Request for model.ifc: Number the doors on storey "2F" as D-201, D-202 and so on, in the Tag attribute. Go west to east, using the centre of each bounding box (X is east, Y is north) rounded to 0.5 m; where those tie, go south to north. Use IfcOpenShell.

First a look at what the model holds.

```python
import ifcopenshell
import ifcopenshell.util.element
import ifcopenshell.util.placement

model = ifcopenshell.open("model.ifc")
print(model.schema)
storey = next(s for s in model.by_type("IfcBuildingStorey") if s.Name == "2F")
doors = [e for e in ifcopenshell.util.element.get_decomposition(storey) if e.is_a("IfcDoor")]
for e in sorted(doors, key=lambda e: e.id()):
    origin = ifcopenshell.util.placement.get_local_placement(e.ObjectPlacement)[:3, 3]
    print(e.id(), e.Tag, e.Name, origin.round(2) + 0.0, sep=" | ")
```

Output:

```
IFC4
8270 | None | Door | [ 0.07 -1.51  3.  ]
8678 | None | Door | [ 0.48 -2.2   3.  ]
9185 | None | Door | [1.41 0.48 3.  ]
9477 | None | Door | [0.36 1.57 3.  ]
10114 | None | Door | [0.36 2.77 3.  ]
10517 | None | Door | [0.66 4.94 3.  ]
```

```python
import ifcopenshell
import ifcopenshell.geom
import ifcopenshell.util.element
import ifcopenshell.util.shape

model = ifcopenshell.open("model.ifc")
settings = ifcopenshell.geom.settings()
settings.set("use-world-coords", True)


def centre(element):
    shape = ifcopenshell.geom.create_shape(settings, element)
    return ifcopenshell.util.shape.get_bbox_centroid(shape.geometry)


storey = next(s for s in model.by_type("IfcBuildingStorey") if s.Name == "2F")
doors = [e for e in ifcopenshell.util.element.get_decomposition(storey) if e.is_a("IfcDoor")]

# Insertion points can sit at a corner or the storey origin, so sort by the geometry (in metres).
centres = {e: centre(e) for e in doors}
doors.sort(key=lambda e: (round(centres[e][0] / 0.5), centres[e][1]))

for i, e in enumerate(doors, start=1):
    number = f"D-2{i:02d}"
    e.Tag = number
    print(e.id(), number)

model.write("model_updated.ifc")
```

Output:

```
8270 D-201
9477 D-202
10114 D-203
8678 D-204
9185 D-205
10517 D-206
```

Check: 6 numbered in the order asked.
